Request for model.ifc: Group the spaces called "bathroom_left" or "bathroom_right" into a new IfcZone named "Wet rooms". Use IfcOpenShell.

First a look at what the model holds.

```python
import ifcopenshell

model = ifcopenshell.open("model.ifc")
print(model.schema)
seen = {}
for space in model.by_type("IfcSpace"):
    seen[space.LongName] = seen.get(space.LongName, 0) + 1
for name, count in sorted(seen.items(), key=str):
    print(count, "x", name)
print("zones:", [z.Name for z in model.by_type("IfcZone")][:20])
```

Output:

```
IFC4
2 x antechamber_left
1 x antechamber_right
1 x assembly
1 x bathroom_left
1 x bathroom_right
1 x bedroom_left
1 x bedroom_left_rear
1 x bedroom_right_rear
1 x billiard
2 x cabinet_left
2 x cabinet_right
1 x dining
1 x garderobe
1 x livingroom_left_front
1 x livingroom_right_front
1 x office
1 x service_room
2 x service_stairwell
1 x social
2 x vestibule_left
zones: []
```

```python
import ifcopenshell
import ifcopenshell.api.group
import ifcopenshell.api.root

model = ifcopenshell.open("model.ifc")

names = {"bathroom_left", "bathroom_right"}
spaces = [s for s in model.by_type("IfcSpace") if s.LongName in names]

zone = ifcopenshell.api.root.create_entity(model, ifc_class="IfcZone", name="Wet rooms")
ifcopenshell.api.group.assign_group(model, products=spaces, group=zone)
print(len(spaces), "spaces in", zone.Name)

model.write("model-out.ifc")
```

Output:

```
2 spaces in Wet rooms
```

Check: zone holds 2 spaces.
